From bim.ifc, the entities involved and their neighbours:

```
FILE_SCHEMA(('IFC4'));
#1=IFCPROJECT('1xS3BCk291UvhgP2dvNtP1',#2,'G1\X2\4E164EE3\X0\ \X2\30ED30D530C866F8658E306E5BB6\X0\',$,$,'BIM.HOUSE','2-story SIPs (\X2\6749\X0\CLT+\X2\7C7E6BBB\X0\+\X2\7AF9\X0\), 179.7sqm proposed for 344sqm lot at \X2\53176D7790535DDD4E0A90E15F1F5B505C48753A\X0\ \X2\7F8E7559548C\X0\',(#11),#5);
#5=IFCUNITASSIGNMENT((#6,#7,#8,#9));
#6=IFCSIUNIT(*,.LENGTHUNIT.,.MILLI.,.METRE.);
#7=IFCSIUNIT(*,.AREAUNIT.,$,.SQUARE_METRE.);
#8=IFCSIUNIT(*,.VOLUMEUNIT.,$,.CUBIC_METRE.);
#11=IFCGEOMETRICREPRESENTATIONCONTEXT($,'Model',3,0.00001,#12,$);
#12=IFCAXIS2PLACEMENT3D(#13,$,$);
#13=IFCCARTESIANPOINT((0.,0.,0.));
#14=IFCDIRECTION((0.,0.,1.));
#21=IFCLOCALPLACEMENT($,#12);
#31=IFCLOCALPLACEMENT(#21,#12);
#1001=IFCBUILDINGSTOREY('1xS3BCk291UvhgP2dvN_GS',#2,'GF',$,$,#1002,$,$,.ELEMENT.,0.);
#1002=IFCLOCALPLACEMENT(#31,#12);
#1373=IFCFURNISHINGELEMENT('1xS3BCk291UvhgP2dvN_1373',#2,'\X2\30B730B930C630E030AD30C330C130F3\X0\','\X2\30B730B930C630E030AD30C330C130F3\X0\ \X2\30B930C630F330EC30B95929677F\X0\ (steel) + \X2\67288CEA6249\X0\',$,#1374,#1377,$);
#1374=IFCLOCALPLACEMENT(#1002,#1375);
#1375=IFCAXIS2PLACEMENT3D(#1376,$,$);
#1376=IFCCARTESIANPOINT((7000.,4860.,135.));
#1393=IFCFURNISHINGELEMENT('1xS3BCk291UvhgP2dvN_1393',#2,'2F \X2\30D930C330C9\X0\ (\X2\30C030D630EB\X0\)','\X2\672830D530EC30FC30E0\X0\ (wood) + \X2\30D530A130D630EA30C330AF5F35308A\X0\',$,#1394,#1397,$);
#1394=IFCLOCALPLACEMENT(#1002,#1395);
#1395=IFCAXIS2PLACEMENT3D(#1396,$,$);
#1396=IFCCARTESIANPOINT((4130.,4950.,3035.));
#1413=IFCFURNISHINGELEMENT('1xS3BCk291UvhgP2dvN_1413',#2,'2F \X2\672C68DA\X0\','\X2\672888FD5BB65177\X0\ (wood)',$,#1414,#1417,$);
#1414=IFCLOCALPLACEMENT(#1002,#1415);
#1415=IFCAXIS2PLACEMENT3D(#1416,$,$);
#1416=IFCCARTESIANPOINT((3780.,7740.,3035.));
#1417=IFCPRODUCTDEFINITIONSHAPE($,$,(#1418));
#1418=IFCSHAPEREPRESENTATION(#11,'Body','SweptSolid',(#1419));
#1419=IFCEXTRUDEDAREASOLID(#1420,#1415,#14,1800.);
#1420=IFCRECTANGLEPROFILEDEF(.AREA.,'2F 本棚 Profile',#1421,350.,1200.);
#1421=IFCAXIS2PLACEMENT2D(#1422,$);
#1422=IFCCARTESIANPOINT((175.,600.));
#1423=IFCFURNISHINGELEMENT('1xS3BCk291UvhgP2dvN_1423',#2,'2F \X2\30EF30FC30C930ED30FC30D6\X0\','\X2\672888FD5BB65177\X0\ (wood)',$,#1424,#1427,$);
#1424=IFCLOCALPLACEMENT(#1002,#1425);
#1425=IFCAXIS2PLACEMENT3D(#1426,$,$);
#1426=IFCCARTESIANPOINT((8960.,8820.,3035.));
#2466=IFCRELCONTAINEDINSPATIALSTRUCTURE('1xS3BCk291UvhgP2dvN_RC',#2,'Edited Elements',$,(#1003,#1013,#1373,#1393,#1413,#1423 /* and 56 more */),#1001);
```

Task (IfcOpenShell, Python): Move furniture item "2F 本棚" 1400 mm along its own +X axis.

```python
import ifcopenshell
import ifcopenshell.api.geometry
import ifcopenshell.util.placement
import ifcopenshell.util.unit

model = ifcopenshell.open("bim.ifc")
unit_scale = ifcopenshell.util.unit.calculate_unit_scale(model)

item = model.by_id(1413)
matrix = ifcopenshell.util.placement.get_local_placement(item.ObjectPlacement)
matrix[:3, 3] += matrix[:3, 0] * 1.4 / unit_scale
ifcopenshell.api.geometry.edit_object_placement(model, product=item, matrix=matrix, is_si=False)

print(ifcopenshell.util.placement.get_local_placement(item.ObjectPlacement).round(3) + 0.0)

model.write("bim_edited.ifc")
```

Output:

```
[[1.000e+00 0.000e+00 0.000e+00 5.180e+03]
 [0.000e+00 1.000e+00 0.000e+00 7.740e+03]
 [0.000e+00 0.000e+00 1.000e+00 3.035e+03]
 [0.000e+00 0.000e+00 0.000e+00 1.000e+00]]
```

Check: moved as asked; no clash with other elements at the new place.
